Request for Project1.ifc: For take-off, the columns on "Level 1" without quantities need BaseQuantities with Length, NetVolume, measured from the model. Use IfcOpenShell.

First a look at what the model holds.

```python
import ifcopenshell
import ifcopenshell.util.element
import ifcopenshell.util.unit

model = ifcopenshell.open("Project1.ifc")
print(model.schema)
for unit_type in ("LENGTHUNIT", "AREAUNIT", "VOLUMEUNIT"):
    print(unit_type, ifcopenshell.util.unit.calculate_unit_scale(model, unit_type))
storey = next(s for s in model.by_type("IfcBuildingStorey") if s.Name == "Level 1")
columns = [e for e in ifcopenshell.util.element.get_decomposition(storey) if e.is_a("IfcColumn")]
for e in sorted(columns, key=lambda e: e.id()):
    print(e.id(), e.is_a(), e.Name, list(ifcopenshell.util.element.get_psets(e, qtos_only=True)), sep=" | ")
```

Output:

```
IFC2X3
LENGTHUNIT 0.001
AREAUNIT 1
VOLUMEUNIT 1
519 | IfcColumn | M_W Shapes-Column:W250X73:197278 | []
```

```python
import ifcopenshell
import ifcopenshell.api.pset
import ifcopenshell.geom
import ifcopenshell.util.element
import ifcopenshell.util.shape
import ifcopenshell.util.unit

model = ifcopenshell.open("Project1.ifc")
unit_scale = ifcopenshell.util.unit.calculate_unit_scale(model)
volume_scale = ifcopenshell.util.unit.calculate_unit_scale(model, "VOLUMEUNIT")
settings = ifcopenshell.geom.settings()

storey = next(s for s in model.by_type("IfcBuildingStorey") if s.Name == "Level 1")
columns = [e for e in ifcopenshell.util.element.get_decomposition(storey) if e.is_a("IfcColumn")]

for e in sorted(columns, key=lambda e: e.id()):
    if ifcopenshell.util.element.get_psets(e, qtos_only=True, should_inherit=False):
        continue
    # Geometry comes back in metres, in the element's own axes.
    shape = ifcopenshell.geom.create_shape(settings, e)
    values = {
        "Length": ifcopenshell.util.shape.get_z(shape.geometry) / unit_scale,
        "NetVolume": ifcopenshell.util.shape.get_volume(shape.geometry) / volume_scale,
    }
    qto = ifcopenshell.api.pset.add_qto(model, product=e, name="BaseQuantities")
    ifcopenshell.api.pset.edit_qto(model, qto=qto, properties=values)
    print(e.id(), {k: round(v, 3) for k, v in values.items()})

model.write("Project1_v2.ifc")
```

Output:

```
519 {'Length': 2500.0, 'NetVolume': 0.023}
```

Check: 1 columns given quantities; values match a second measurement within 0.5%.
